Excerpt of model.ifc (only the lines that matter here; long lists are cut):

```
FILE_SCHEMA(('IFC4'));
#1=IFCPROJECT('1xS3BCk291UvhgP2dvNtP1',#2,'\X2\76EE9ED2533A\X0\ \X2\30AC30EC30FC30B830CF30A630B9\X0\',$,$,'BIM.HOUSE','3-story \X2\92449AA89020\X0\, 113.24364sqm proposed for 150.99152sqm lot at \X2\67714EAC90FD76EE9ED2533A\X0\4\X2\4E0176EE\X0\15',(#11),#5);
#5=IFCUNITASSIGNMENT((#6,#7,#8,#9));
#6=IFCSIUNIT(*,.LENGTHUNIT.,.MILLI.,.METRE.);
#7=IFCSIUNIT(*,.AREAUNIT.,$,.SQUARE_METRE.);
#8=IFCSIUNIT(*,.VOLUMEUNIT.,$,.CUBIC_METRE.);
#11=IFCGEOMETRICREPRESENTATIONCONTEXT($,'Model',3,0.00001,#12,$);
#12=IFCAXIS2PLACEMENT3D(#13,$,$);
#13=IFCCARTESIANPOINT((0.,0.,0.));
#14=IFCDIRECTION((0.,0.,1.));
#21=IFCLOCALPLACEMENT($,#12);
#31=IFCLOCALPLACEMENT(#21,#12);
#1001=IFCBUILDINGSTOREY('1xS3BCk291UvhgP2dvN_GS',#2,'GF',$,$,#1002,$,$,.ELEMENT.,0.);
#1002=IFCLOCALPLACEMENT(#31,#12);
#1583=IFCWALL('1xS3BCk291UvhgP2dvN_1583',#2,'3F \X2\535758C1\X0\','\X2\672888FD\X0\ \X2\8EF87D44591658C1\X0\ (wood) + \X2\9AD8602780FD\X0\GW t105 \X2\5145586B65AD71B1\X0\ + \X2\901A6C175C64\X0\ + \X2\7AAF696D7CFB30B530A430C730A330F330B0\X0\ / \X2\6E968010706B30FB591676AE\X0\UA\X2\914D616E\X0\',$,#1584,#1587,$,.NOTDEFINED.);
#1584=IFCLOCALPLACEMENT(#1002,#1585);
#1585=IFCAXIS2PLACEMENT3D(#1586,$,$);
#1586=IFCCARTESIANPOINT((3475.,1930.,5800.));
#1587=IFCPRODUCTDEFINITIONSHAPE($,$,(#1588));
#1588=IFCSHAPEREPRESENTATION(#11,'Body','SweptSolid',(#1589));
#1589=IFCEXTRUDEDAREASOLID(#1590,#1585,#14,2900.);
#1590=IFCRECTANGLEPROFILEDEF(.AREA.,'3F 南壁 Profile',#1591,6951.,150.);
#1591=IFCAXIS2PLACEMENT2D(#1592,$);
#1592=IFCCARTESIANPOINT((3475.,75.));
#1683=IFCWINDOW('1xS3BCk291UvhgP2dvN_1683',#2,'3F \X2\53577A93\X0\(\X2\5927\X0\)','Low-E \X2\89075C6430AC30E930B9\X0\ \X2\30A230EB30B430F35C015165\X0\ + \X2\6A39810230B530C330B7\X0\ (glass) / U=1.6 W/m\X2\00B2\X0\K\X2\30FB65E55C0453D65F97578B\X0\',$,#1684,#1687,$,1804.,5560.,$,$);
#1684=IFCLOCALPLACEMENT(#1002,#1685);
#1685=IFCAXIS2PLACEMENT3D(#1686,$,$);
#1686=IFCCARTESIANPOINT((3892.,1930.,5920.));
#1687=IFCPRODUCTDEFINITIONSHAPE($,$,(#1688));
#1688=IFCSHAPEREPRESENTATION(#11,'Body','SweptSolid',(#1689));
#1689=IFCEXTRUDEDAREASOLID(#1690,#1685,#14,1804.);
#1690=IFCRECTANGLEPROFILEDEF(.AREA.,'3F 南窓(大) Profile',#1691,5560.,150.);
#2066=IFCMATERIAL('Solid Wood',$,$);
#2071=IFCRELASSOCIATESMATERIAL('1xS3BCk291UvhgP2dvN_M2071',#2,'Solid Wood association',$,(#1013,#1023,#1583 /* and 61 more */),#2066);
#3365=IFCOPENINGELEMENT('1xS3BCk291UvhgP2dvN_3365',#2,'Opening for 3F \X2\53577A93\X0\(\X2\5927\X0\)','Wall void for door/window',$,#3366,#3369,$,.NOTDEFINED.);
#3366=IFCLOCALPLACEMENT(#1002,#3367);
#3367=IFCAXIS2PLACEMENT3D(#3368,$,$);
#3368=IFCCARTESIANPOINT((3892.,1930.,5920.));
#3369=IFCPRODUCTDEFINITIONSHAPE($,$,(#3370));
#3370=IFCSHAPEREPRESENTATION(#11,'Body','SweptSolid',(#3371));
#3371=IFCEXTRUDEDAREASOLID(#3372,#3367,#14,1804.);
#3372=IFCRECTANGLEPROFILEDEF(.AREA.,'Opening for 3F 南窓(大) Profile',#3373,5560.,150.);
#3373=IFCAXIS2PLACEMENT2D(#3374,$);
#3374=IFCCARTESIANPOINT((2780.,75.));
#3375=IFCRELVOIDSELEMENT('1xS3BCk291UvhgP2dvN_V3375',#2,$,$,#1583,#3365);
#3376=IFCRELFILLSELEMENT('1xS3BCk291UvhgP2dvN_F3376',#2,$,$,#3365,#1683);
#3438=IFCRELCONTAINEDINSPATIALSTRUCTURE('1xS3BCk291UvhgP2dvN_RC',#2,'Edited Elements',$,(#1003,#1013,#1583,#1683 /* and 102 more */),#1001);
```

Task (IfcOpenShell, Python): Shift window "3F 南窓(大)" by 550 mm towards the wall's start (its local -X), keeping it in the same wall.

```python
import ifcopenshell
import ifcopenshell.api.geometry
import ifcopenshell.util.placement
import ifcopenshell.util.unit

model = ifcopenshell.open("model.ifc")
unit_scale = ifcopenshell.util.unit.calculate_unit_scale(model)

window = model.by_guid("1xS3BCk291UvhgP2dvN_1683")
opening = window.FillsVoids[0].RelatingOpeningElement
wall = opening.VoidsElements[0].RelatingBuildingElement

wall_matrix = ifcopenshell.util.placement.get_local_placement(wall.ObjectPlacement)
shift = wall_matrix[:3, 0] * -0.55 / unit_scale
before = ifcopenshell.util.placement.get_local_placement(window.ObjectPlacement)[:3, 3].copy()

# The window is not placed relative to its opening, so move both.
for product in (opening, window):
    matrix = ifcopenshell.util.placement.get_local_placement(product.ObjectPlacement)
    matrix[:3, 3] += shift
    ifcopenshell.api.geometry.edit_object_placement(model, product=product, matrix=matrix, is_si=False)

after = ifcopenshell.util.placement.get_local_placement(window.ObjectPlacement)[:3, 3]
print("window moved by", (after - before).round(3) + 0.0)

model.write("model_v2.ifc")
```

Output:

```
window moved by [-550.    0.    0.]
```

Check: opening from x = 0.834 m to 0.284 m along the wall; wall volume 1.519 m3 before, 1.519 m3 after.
